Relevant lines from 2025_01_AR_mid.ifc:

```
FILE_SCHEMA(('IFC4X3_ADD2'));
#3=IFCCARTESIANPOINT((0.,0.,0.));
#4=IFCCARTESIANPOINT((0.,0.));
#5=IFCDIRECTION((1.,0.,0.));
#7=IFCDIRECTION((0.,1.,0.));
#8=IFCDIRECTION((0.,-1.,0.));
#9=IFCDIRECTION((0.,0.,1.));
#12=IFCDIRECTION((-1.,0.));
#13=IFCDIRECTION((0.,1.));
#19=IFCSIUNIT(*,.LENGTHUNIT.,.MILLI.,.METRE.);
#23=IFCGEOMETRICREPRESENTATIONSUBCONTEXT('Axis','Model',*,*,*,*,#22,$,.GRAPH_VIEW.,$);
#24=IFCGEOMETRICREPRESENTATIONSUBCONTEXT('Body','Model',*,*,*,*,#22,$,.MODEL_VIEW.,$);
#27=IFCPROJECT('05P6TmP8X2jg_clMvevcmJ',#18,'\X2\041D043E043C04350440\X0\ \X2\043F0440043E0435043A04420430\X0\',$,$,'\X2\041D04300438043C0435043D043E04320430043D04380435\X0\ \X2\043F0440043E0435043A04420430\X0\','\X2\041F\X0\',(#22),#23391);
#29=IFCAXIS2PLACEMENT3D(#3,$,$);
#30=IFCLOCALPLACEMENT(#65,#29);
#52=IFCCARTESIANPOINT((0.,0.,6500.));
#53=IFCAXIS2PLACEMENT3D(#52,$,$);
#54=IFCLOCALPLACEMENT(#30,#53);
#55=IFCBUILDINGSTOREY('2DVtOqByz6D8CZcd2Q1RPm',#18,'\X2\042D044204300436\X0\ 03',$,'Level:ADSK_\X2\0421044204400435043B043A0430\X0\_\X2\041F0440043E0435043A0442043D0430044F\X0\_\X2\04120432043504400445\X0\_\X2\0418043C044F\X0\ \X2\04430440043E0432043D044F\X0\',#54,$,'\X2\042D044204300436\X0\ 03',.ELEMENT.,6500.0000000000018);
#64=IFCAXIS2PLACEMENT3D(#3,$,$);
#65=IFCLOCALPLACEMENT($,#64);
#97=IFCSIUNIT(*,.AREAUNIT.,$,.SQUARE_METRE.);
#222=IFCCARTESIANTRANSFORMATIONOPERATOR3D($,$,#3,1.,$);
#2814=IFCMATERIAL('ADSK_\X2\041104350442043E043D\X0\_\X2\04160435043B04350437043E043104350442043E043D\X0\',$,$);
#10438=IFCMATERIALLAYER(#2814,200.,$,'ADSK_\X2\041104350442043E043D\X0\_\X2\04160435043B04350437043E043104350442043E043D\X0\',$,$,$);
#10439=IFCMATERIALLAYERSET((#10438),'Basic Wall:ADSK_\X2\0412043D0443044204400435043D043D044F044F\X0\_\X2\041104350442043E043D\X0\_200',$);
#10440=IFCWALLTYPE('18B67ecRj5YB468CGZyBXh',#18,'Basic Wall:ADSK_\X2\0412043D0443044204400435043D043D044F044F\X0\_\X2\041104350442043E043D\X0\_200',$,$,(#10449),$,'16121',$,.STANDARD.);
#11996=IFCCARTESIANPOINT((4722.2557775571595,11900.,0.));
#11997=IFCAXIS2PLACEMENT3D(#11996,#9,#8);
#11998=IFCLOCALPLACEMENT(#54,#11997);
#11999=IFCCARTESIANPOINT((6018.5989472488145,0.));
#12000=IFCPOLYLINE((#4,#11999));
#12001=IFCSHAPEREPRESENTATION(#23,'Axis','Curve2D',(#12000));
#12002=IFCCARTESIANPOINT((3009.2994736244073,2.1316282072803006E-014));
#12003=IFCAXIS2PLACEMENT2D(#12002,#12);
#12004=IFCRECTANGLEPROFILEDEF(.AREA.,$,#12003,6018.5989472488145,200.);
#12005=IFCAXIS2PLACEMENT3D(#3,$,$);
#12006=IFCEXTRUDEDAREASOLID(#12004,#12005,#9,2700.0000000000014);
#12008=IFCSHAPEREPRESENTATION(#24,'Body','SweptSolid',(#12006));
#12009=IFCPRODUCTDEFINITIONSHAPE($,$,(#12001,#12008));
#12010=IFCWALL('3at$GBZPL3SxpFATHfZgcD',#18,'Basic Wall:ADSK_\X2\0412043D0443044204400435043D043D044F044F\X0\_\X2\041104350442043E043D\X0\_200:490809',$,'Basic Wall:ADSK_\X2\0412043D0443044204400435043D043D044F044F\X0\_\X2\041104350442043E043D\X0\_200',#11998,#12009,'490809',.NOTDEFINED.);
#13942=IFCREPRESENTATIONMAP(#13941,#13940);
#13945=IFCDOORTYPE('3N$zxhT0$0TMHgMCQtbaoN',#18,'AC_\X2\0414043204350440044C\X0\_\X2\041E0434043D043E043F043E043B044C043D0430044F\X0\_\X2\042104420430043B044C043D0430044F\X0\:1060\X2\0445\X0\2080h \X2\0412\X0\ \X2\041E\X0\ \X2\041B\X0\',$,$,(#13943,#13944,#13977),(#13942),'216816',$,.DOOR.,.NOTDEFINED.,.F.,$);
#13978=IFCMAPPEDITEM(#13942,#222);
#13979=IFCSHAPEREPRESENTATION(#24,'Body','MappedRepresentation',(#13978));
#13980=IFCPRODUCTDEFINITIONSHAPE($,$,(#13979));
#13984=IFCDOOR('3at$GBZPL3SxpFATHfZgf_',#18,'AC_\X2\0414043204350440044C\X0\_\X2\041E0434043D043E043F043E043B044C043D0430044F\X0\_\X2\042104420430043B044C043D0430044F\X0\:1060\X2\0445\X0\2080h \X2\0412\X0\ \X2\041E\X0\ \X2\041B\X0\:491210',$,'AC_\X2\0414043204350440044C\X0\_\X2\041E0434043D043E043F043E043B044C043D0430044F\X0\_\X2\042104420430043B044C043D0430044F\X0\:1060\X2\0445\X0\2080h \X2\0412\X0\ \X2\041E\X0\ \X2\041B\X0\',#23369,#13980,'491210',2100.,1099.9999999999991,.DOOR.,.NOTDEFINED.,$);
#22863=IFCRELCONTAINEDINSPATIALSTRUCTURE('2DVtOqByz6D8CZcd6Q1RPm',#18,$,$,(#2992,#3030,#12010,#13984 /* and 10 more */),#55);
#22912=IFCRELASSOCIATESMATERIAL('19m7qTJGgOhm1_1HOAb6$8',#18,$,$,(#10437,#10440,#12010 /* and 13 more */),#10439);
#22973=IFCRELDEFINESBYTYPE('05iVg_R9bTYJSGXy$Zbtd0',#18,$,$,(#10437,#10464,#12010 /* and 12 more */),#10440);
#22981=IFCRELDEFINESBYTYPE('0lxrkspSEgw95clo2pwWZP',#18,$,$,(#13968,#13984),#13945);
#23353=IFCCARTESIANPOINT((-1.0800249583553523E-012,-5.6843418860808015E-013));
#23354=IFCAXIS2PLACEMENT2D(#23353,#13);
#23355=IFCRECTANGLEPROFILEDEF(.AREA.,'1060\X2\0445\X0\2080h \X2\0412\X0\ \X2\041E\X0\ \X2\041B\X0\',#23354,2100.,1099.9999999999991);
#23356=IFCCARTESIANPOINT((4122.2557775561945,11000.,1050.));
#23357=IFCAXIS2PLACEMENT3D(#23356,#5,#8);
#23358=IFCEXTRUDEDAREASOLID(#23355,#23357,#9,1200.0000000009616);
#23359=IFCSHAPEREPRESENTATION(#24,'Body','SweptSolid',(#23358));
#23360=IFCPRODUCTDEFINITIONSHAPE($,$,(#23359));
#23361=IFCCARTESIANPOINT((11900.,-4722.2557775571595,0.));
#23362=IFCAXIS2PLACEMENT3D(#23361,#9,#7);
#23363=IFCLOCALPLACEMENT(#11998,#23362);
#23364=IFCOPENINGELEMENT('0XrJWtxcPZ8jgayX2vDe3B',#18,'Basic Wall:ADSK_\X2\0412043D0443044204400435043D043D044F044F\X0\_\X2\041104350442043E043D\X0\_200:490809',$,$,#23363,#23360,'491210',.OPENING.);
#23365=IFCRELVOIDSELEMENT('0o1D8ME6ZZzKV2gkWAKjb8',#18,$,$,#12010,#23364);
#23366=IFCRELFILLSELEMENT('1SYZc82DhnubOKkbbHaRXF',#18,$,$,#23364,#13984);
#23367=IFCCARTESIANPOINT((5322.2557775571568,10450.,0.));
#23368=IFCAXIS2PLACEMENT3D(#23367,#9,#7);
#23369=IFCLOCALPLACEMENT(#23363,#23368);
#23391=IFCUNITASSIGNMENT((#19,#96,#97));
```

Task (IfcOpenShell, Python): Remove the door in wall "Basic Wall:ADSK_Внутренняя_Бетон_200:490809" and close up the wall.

```python
import ifcopenshell
import ifcopenshell.api.feature
import ifcopenshell.api.root
import ifcopenshell.geom
import ifcopenshell.util.shape

model = ifcopenshell.open("2025_01_AR_mid.ifc")
settings = ifcopenshell.geom.settings()


def volume(element):
    """Net volume in cubic metres, openings subtracted."""
    shape = ifcopenshell.geom.create_shape(settings, element)
    return ifcopenshell.util.shape.get_volume(shape.geometry)


door = model.by_id(13984)
opening = door.FillsVoids[0].RelatingOpeningElement
wall = opening.VoidsElements[0].RelatingBuildingElement
before = volume(wall)

ifcopenshell.api.root.remove_product(model, product=door)
ifcopenshell.api.feature.remove_feature(model, feature=opening)

after = volume(wall)

print(f"wall volume {before:.3f} -> {after:.3f} m3")

model.write("2025_01_AR_mid_v2.ifc")
```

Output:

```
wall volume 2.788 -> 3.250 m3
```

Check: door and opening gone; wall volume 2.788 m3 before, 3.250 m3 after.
